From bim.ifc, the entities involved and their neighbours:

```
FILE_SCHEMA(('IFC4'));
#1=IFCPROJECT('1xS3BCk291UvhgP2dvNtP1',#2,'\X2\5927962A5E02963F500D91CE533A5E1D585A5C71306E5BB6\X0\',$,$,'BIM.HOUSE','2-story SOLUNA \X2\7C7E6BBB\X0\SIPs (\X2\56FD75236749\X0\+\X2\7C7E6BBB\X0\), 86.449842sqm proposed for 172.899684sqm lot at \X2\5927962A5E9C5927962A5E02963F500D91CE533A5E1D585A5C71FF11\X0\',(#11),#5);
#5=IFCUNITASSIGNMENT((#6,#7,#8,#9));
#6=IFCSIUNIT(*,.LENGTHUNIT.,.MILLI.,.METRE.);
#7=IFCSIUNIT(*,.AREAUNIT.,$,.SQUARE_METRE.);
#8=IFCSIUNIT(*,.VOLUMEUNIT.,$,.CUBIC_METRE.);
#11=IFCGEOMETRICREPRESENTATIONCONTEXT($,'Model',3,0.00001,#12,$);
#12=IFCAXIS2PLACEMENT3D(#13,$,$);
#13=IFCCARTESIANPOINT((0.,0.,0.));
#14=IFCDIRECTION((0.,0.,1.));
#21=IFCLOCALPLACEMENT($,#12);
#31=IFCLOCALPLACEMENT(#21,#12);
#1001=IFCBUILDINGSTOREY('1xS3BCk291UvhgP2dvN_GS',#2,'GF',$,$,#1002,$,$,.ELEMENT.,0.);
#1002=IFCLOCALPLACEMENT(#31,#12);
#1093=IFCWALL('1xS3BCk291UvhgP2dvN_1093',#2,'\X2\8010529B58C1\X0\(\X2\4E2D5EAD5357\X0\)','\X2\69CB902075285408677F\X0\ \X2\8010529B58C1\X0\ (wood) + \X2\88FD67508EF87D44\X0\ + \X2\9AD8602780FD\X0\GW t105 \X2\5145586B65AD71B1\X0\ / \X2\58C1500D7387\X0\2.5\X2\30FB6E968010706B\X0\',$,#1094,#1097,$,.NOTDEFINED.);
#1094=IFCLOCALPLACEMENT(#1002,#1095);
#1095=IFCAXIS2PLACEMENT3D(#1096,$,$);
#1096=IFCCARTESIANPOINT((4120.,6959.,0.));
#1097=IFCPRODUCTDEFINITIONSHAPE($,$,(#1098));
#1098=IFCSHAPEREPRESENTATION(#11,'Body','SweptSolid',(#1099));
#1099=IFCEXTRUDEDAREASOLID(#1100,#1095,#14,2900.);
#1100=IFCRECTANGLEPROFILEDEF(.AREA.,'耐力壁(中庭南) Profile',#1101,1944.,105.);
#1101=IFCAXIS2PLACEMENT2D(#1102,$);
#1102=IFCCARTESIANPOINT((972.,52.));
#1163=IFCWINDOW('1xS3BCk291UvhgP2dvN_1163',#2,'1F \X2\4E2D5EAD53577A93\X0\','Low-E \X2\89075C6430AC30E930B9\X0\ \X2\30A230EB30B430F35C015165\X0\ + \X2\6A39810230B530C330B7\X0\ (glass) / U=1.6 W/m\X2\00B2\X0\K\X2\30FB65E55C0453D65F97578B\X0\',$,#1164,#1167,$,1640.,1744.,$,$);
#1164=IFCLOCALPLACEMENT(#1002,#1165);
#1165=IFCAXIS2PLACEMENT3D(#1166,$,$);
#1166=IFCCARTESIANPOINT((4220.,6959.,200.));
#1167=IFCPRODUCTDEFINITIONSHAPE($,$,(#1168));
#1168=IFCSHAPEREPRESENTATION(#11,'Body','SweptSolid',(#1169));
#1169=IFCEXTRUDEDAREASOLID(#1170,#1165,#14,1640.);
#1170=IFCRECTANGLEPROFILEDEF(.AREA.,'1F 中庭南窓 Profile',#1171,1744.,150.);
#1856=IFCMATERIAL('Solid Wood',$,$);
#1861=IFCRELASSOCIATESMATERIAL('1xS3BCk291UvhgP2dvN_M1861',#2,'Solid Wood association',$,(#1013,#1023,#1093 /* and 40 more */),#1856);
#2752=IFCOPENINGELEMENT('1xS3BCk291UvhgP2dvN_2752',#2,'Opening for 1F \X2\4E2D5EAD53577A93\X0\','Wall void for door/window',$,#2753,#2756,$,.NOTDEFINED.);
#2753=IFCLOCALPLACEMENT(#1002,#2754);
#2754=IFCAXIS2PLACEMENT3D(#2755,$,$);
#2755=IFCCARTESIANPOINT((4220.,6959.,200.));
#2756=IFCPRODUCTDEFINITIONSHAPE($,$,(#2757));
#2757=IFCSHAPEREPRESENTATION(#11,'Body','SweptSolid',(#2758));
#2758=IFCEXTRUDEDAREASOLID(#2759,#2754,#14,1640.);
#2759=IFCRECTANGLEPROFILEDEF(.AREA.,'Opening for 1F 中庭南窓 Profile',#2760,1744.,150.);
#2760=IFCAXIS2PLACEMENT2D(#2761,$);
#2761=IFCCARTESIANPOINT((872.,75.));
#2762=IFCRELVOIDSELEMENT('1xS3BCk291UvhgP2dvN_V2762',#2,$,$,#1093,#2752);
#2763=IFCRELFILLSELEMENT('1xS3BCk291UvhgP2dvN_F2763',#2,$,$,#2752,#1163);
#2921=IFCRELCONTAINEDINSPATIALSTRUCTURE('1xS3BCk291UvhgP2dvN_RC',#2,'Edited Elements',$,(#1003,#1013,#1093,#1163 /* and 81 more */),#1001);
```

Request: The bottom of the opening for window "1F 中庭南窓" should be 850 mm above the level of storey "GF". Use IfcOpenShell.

```python
import numpy as np
import ifcopenshell
import ifcopenshell.api.geometry
import ifcopenshell.geom
import ifcopenshell.util.element
import ifcopenshell.util.placement
import ifcopenshell.util.shape
import ifcopenshell.util.unit

model = ifcopenshell.open("bim.ifc")
unit_scale = ifcopenshell.util.unit.calculate_unit_scale(model)

window = model.by_guid("1xS3BCk291UvhgP2dvN_1163")
opening = window.FillsVoids[0].RelatingOpeningElement
storey = ifcopenshell.util.element.get_container(window, ifc_class="IfcBuildingStorey")
level = ifcopenshell.util.placement.get_local_placement(storey.ObjectPlacement)[2, 3]

# The opening's origin need not be at the sill, so measure its lowest point.
shape = ifcopenshell.geom.create_shape(ifcopenshell.geom.settings(), opening)
bottom = ifcopenshell.util.shape.get_shape_bottom_elevation(shape, shape.geometry) / unit_scale
dz = level + 850.0 - bottom

shift = np.array([0.0, 0.0, dz])
# The window is not placed relative to its opening, so move both.
for product in (opening, window):
    matrix = ifcopenshell.util.placement.get_local_placement(product.ObjectPlacement)
    matrix[:3, 3] += shift
    ifcopenshell.api.geometry.edit_object_placement(model, product=product, matrix=matrix, is_si=False)

print(f"moved by {dz * unit_scale:+.3f} m")

model.write("bim_edited.ifc")
```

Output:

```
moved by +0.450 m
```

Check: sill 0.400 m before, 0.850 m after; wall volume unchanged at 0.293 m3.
